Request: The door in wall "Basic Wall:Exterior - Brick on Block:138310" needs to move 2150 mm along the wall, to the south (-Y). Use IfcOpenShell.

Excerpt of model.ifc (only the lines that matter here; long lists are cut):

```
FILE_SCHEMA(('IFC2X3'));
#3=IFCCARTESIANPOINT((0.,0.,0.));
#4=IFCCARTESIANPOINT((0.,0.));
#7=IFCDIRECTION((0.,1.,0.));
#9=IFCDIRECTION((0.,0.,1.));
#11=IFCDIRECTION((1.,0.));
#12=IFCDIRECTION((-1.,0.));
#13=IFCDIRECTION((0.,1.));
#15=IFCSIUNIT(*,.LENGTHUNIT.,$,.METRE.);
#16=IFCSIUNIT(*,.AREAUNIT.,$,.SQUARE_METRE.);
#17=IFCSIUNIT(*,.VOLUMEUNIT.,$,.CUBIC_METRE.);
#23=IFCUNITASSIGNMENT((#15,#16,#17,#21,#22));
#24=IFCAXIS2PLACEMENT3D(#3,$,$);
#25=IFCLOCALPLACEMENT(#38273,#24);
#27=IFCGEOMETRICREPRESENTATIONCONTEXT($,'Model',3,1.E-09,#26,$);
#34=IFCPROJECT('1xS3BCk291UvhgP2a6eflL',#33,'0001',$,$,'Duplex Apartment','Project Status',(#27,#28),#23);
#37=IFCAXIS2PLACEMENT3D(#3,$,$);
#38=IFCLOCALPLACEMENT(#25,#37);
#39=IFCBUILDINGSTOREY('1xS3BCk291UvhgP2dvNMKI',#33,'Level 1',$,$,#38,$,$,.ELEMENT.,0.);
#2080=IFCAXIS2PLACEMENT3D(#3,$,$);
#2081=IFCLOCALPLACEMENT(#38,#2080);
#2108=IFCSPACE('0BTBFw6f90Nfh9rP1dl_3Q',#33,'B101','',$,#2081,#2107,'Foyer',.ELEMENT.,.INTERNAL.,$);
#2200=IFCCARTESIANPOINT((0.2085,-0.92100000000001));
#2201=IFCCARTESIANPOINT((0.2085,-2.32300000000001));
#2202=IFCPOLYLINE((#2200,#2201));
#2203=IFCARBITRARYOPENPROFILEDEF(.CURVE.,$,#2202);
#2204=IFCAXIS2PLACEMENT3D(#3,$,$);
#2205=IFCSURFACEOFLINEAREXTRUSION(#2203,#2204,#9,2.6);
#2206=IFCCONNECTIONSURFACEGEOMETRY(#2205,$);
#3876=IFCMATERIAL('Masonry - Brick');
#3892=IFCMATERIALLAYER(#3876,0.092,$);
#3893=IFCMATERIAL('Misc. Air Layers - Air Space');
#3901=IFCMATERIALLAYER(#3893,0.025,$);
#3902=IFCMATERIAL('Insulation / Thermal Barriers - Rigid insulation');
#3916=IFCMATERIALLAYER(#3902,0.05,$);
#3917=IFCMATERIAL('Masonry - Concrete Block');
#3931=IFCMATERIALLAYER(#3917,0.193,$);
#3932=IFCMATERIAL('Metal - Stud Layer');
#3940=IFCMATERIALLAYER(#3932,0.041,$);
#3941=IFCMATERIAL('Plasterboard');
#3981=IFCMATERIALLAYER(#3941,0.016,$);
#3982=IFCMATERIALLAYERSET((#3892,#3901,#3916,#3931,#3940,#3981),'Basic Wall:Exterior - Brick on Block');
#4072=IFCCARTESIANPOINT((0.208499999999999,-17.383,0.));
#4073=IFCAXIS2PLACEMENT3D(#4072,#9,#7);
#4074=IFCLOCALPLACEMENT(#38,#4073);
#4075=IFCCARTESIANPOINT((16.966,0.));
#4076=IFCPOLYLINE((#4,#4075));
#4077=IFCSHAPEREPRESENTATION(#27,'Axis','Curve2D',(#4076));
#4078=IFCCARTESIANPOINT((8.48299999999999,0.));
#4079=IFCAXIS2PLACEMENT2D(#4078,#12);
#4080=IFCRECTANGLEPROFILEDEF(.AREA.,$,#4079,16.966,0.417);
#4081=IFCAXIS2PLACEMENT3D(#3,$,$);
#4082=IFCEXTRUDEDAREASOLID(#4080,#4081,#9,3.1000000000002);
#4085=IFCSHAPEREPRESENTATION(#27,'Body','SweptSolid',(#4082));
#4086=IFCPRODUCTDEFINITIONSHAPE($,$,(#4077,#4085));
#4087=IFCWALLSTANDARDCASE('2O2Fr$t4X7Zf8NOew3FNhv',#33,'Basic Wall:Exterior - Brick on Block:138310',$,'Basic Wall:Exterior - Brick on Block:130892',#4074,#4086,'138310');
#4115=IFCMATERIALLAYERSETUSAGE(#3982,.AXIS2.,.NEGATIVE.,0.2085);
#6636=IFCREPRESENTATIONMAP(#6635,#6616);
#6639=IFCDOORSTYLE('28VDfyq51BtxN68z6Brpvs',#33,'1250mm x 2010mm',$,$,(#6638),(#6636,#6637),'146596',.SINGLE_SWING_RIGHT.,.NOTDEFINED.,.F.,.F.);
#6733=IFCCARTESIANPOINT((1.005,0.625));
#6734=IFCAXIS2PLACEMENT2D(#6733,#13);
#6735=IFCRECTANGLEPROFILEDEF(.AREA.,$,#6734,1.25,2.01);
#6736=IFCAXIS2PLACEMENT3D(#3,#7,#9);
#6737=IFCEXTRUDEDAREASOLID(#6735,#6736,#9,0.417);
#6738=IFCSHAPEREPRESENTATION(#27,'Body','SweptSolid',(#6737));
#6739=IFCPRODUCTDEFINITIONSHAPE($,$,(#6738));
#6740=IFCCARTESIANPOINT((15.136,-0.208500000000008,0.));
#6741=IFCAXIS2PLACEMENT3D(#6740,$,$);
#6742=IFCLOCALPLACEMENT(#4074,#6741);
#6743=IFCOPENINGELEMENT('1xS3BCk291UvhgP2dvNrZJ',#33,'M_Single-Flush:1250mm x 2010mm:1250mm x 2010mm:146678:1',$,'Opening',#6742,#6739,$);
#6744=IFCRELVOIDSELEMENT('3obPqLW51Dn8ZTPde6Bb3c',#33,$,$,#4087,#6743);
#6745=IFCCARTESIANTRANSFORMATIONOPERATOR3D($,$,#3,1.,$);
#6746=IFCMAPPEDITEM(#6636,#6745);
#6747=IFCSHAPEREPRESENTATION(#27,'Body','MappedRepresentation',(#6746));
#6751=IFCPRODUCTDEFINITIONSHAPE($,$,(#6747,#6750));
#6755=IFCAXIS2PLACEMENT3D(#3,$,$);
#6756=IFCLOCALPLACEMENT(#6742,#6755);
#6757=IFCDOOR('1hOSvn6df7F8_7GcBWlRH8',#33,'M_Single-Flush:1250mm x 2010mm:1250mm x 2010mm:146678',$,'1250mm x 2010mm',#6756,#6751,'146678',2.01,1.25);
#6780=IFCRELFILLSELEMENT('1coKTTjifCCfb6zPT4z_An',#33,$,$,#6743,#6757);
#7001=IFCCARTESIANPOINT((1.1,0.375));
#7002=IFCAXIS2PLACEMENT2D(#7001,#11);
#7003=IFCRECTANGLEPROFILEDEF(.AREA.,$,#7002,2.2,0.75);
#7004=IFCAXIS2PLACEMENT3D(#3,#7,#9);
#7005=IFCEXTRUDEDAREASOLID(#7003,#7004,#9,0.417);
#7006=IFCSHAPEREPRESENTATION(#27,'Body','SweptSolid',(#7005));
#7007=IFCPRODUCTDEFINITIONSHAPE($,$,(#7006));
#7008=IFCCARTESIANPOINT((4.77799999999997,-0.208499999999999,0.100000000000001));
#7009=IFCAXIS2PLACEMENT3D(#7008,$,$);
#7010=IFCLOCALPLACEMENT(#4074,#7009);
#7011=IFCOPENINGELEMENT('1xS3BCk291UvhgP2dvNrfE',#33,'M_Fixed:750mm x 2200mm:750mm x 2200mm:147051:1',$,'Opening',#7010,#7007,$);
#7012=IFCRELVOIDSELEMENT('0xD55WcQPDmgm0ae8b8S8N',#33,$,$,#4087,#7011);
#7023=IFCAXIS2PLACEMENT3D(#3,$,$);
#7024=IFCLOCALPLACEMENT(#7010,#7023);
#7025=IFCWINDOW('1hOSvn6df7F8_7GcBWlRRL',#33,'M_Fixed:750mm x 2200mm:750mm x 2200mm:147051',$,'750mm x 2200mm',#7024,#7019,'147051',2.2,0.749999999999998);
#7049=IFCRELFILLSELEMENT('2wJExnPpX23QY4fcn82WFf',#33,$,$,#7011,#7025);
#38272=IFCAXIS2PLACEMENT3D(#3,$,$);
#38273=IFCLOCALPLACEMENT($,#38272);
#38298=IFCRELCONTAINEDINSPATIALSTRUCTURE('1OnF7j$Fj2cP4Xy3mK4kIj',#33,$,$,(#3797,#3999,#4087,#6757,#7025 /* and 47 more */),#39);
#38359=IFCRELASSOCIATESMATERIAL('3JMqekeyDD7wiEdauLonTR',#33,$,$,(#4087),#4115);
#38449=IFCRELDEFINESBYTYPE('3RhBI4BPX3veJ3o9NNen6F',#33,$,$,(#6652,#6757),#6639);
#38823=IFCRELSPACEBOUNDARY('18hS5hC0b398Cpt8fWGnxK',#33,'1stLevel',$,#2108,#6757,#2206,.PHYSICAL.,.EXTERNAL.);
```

```python
import numpy as np
import ifcopenshell
import ifcopenshell.api.geometry
import ifcopenshell.util.placement

model = ifcopenshell.open("model.ifc")

door = model.by_guid("1hOSvn6df7F8_7GcBWlRH8")
opening = door.FillsVoids[0].RelatingOpeningElement
wall = opening.VoidsElements[0].RelatingBuildingElement

wall_matrix = ifcopenshell.util.placement.get_local_placement(wall.ObjectPlacement)
shift = wall_matrix[:3, 0] * -2.15
before = ifcopenshell.util.placement.get_local_placement(door.ObjectPlacement)[:3, 3].copy()

# The door is placed relative to its opening, so it follows when the opening moves.
matrix = ifcopenshell.util.placement.get_local_placement(opening.ObjectPlacement)
matrix[:3, 3] += shift
ifcopenshell.api.geometry.edit_object_placement(
    model, product=opening, matrix=matrix, is_si=False, should_transform_children=True
)

# Space boundary surfaces are stored in each space's coordinates; move them too.
for rel in door.ProvidesBoundaries:
    if not rel.ConnectionGeometry:
        continue
    surface = rel.ConnectionGeometry.SurfaceOnRelatingElement
    space_matrix = ifcopenshell.util.placement.get_local_placement(rel.RelatingSpace.ObjectPlacement)
    point = np.array(surface.Position.Location.Coordinates) + space_matrix[:3, :3].T @ shift
    surface.Position = model.createIfcAxis2Placement3D(
        model.createIfcCartesianPoint(point.tolist()), surface.Position.Axis, surface.Position.RefDirection
    )

after = ifcopenshell.util.placement.get_local_placement(door.ObjectPlacement)[:3, 3]
print("door moved by", (after - before).round(3) + 0.0)

model.write("model_updated.ifc")
```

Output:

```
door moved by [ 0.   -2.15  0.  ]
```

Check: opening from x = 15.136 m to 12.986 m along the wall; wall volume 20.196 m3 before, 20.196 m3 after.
